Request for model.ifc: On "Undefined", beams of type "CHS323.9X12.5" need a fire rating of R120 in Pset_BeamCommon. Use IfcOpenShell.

First a look at what the model holds.

```python
import ifcopenshell
import ifcopenshell.util.element

model = ifcopenshell.open("model.ifc")
print(model.schema)
storey = next(s for s in model.by_type("IfcBuildingStorey") if s.Name == "Undefined")
beams = [e for e in ifcopenshell.util.element.get_decomposition(storey) if e.is_a("IfcBeam")]
seen = {}
for e in beams:
    element_type = ifcopenshell.util.element.get_type(e)
    key = (element_type.Name if element_type != e and element_type else None, ifcopenshell.util.element.get_pset(e, "Pset_BeamCommon", "FireRating"))
    seen[key] = seen.get(key, 0) + 1
for (name, value), count in sorted(seen.items(), key=str):
    print(count, "x", name, "|", value)
```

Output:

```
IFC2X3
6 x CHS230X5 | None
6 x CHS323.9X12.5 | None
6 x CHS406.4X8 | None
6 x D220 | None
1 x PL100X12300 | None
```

```python
import ifcopenshell
import ifcopenshell.api.pset
import ifcopenshell.util.element

model = ifcopenshell.open("model.ifc")

storey = next(s for s in model.by_type("IfcBuildingStorey") if s.Name == "Undefined")
beams = [e for e in ifcopenshell.util.element.get_decomposition(storey) if e.is_a("IfcBeam")]

count = 0
for e in beams:
    element_type = ifcopenshell.util.element.get_type(e)
    if element_type in (None, e) or element_type.Name != "CHS323.9X12.5":
        continue
    found = ifcopenshell.util.element.get_pset(e, "Pset_BeamCommon", should_inherit=False)
    if found:
        pset = model.by_id(found["id"])
        if len(ifcopenshell.util.element.get_elements_by_pset(pset)) > 1:
            pset = ifcopenshell.api.pset.unshare_pset(model, products=[e], pset=pset)[0]
    else:
        pset = ifcopenshell.api.pset.add_pset(model, product=e, name="Pset_BeamCommon")
    ifcopenshell.api.pset.edit_pset(model, pset=pset, properties={"FireRating": "R120"})
    count += 1

print(count, "beams updated")

model.write("model-out.ifc")
```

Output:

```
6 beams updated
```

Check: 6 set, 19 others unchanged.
